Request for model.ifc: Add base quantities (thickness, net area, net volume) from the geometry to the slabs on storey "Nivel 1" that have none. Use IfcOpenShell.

First a look at what the model holds.

```python
import ifcopenshell
import ifcopenshell.util.element
import ifcopenshell.util.unit

model = ifcopenshell.open("model.ifc")
print(model.schema)
for unit_type in ("LENGTHUNIT", "AREAUNIT", "VOLUMEUNIT"):
    print(unit_type, ifcopenshell.util.unit.calculate_unit_scale(model, unit_type))
storey = next(s for s in model.by_type("IfcBuildingStorey") if s.Name == "Nivel 1")
slabs = [e for e in ifcopenshell.util.element.get_decomposition(storey) if e.is_a("IfcSlab")]
for e in sorted(slabs, key=lambda e: e.id()):
    print(e.id(), e.is_a(), e.Name, list(ifcopenshell.util.element.get_psets(e, qtos_only=True)), sep=" | ")
```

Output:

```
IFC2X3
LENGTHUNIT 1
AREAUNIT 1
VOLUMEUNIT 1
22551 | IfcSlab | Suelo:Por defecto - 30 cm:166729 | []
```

```python
import ifcopenshell
import ifcopenshell.api.pset
import ifcopenshell.geom
import ifcopenshell.util.element
import ifcopenshell.util.shape
import ifcopenshell.util.unit

model = ifcopenshell.open("model.ifc")
unit_scale = ifcopenshell.util.unit.calculate_unit_scale(model)
area_scale = ifcopenshell.util.unit.calculate_unit_scale(model, "AREAUNIT")
volume_scale = ifcopenshell.util.unit.calculate_unit_scale(model, "VOLUMEUNIT")
settings = ifcopenshell.geom.settings()

storey = next(s for s in model.by_type("IfcBuildingStorey") if s.Name == "Nivel 1")
slabs = [e for e in ifcopenshell.util.element.get_decomposition(storey) if e.is_a("IfcSlab")]

for e in sorted(slabs, key=lambda e: e.id()):
    if ifcopenshell.util.element.get_psets(e, qtos_only=True, should_inherit=False):
        continue
    # Geometry comes back in metres, in the element's own axes.
    shape = ifcopenshell.geom.create_shape(settings, e)
    values = {
        "Width": ifcopenshell.util.shape.get_z(shape.geometry) / unit_scale,
        "NetArea": ifcopenshell.util.shape.get_footprint_area(shape.geometry) / area_scale,
        "NetVolume": ifcopenshell.util.shape.get_volume(shape.geometry) / volume_scale,
    }
    qto = ifcopenshell.api.pset.add_qto(model, product=e, name="BaseQuantities")
    ifcopenshell.api.pset.edit_qto(model, qto=qto, properties=values)
    print(e.id(), {k: round(v, 3) for k, v in values.items()})

model.write("model-out.ifc")
```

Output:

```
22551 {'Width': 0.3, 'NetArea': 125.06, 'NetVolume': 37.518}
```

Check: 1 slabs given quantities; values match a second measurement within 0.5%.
